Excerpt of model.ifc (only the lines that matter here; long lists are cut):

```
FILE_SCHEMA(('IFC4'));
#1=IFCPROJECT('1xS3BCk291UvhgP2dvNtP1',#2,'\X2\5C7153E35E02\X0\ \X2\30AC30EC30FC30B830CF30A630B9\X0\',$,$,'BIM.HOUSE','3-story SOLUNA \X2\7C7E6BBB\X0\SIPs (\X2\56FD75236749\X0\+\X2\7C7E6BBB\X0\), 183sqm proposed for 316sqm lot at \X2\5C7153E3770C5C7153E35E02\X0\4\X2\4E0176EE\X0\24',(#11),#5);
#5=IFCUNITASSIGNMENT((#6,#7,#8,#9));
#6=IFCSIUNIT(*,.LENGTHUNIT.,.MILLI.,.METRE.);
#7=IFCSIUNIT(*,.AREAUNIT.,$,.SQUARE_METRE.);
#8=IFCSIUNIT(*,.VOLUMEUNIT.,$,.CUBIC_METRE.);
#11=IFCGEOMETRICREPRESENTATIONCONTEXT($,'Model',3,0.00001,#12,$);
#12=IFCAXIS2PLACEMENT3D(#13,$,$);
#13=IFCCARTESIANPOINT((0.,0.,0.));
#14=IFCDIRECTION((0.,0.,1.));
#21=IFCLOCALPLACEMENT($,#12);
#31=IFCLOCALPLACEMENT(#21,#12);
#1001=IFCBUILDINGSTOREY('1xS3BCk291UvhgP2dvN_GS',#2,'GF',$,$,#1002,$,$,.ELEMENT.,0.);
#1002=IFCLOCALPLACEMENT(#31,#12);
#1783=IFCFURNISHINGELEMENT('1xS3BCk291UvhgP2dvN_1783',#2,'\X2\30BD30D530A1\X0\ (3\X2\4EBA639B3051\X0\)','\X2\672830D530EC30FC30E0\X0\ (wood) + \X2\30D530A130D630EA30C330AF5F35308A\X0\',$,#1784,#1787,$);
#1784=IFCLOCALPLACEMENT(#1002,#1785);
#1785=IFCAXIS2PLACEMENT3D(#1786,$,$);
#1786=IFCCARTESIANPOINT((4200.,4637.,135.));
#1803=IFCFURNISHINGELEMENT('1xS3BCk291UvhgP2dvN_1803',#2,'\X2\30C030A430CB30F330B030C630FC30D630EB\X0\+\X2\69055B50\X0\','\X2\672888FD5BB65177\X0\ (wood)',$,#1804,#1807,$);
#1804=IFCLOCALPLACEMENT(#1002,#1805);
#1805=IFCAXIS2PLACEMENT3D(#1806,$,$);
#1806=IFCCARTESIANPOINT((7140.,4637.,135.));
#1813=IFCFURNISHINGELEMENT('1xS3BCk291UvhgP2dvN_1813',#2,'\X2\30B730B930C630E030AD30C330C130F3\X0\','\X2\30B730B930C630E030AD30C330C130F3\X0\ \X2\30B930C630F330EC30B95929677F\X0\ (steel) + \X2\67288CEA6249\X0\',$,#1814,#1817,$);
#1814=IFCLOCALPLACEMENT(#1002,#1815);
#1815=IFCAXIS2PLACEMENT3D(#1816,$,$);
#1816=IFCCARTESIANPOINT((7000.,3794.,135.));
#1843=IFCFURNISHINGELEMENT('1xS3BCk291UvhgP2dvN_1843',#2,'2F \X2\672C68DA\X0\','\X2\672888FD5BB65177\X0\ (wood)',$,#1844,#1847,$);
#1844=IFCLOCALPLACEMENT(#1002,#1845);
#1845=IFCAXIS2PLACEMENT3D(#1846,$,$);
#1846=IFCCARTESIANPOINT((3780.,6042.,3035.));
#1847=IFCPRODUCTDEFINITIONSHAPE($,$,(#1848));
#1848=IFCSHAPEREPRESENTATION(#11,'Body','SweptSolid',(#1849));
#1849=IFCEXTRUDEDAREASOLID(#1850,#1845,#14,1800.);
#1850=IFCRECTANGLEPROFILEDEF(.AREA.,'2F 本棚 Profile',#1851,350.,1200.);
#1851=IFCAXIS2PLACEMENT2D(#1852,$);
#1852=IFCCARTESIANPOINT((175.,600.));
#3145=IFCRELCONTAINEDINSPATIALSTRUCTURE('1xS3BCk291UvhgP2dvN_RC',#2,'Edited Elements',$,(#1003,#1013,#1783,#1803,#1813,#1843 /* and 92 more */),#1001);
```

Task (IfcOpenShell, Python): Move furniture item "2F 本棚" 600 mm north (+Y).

```python
import ifcopenshell
import ifcopenshell.api.geometry
import ifcopenshell.util.placement

model = ifcopenshell.open("model.ifc")

item = model.by_guid("1xS3BCk291UvhgP2dvN_1843")
matrix = ifcopenshell.util.placement.get_local_placement(item.ObjectPlacement)
matrix[1, 3] += 600.0
ifcopenshell.api.geometry.edit_object_placement(model, product=item, matrix=matrix, is_si=False)

print(ifcopenshell.util.placement.get_local_placement(item.ObjectPlacement).round(3) + 0.0)

model.write("model_edited.ifc")
```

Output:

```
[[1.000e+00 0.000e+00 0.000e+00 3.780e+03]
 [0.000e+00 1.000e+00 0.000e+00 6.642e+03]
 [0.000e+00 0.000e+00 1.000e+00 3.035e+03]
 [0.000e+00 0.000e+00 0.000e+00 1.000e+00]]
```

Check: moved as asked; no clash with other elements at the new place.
